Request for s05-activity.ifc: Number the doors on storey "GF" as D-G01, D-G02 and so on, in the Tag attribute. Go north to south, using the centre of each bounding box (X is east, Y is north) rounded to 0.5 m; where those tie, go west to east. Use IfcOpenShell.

First a look at what the model holds.

```python
import ifcopenshell
import ifcopenshell.util.element
import ifcopenshell.util.placement

model = ifcopenshell.open("s05-activity.ifc")
print(model.schema)
storey = next(s for s in model.by_type("IfcBuildingStorey") if s.Name == "GF")
doors = [e for e in ifcopenshell.util.element.get_decomposition(storey) if e.is_a("IfcDoor")]
for e in sorted(doors, key=lambda e: e.id()):
    origin = ifcopenshell.util.placement.get_local_placement(e.ObjectPlacement)[:3, 3]
    print(e.id(), e.Tag, e.Name, origin.round(2) + 0.0, sep=" | ")
```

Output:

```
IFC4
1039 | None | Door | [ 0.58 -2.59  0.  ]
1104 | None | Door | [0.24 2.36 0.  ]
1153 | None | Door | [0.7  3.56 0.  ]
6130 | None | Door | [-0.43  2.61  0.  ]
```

```python
import ifcopenshell
import ifcopenshell.geom
import ifcopenshell.util.element
import ifcopenshell.util.shape

model = ifcopenshell.open("s05-activity.ifc")
settings = ifcopenshell.geom.settings()
settings.set("use-world-coords", True)


def centre(element):
    shape = ifcopenshell.geom.create_shape(settings, element)
    return ifcopenshell.util.shape.get_bbox_centroid(shape.geometry)


storey = next(s for s in model.by_type("IfcBuildingStorey") if s.Name == "GF")
doors = [e for e in ifcopenshell.util.element.get_decomposition(storey) if e.is_a("IfcDoor")]

# Insertion points can sit at a corner or the storey origin, so sort by the geometry (in metres).
centres = {e: centre(e) for e in doors}
doors.sort(key=lambda e: (-round(centres[e][1] / 0.5), centres[e][0]))

for i, e in enumerate(doors, start=1):
    number = f"D-G{i:02d}"
    e.Tag = number
    print(e.id(), number)

model.write("s05-activity-out.ifc")
```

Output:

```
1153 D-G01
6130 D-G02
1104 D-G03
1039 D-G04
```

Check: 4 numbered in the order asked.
